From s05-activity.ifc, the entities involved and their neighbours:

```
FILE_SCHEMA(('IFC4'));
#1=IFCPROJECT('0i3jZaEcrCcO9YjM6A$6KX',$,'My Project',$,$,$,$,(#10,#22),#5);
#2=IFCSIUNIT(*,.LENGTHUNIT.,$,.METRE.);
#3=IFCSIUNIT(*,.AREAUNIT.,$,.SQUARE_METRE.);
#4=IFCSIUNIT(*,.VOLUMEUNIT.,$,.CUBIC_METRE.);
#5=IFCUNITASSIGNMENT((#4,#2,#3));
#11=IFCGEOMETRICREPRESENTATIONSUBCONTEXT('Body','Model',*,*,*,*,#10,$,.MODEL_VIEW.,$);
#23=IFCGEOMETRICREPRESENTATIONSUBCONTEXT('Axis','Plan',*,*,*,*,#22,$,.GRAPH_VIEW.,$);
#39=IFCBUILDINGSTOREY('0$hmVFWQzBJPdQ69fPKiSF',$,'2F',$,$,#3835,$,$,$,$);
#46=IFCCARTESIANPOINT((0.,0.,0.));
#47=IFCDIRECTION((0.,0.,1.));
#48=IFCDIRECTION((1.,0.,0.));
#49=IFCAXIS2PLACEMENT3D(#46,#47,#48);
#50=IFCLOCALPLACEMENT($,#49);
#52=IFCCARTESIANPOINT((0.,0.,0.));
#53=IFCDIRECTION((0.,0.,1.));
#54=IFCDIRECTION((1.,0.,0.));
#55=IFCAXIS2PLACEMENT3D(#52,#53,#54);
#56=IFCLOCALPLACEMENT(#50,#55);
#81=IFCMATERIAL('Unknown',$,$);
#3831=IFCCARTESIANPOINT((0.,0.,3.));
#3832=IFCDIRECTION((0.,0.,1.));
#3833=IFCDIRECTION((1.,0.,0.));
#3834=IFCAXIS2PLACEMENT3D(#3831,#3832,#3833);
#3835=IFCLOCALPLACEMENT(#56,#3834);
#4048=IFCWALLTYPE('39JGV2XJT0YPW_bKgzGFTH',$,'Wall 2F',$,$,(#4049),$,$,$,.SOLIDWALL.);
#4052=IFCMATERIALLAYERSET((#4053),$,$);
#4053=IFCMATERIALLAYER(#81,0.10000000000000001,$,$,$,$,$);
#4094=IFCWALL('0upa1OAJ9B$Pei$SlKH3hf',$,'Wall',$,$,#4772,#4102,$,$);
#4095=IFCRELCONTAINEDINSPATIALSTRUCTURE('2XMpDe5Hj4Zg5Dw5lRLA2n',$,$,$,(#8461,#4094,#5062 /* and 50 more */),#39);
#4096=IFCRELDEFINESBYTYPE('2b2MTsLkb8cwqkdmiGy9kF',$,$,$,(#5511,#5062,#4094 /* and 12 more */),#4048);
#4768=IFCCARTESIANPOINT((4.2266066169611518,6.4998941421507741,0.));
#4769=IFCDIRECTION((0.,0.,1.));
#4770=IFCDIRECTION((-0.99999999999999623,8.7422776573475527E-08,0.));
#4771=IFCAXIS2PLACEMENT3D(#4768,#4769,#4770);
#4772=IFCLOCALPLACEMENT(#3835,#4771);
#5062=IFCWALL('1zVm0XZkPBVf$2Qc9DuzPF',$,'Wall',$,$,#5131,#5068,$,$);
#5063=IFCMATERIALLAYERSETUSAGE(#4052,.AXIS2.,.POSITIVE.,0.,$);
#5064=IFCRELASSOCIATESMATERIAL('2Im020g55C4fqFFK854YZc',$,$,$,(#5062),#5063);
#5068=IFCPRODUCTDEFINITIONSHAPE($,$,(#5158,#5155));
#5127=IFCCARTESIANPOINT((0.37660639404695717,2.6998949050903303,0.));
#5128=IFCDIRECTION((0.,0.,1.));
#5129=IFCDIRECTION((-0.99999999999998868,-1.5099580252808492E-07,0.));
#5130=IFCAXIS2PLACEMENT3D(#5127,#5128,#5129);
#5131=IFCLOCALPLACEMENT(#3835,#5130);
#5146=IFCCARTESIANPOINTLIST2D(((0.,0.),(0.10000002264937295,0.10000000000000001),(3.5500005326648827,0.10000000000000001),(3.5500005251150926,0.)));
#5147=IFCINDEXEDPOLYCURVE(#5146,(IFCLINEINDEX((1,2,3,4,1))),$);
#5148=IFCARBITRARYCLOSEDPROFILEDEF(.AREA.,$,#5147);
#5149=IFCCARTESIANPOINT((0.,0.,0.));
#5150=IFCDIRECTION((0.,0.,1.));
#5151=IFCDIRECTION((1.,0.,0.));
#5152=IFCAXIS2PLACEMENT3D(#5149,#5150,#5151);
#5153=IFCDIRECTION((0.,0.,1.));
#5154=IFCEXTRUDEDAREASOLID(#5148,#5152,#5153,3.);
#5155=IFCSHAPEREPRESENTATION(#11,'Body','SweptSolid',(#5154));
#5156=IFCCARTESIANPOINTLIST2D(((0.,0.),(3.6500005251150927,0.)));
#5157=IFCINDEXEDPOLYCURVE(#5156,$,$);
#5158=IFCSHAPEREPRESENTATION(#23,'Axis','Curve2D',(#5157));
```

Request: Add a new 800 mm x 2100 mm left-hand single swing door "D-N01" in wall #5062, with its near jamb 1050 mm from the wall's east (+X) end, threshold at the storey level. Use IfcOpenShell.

```python
import numpy as np
import ifcopenshell
import ifcopenshell.api.feature
import ifcopenshell.api.geometry
import ifcopenshell.api.root
import ifcopenshell.api.spatial
import ifcopenshell.geom
import ifcopenshell.util.element
import ifcopenshell.util.placement
import ifcopenshell.util.representation
import ifcopenshell.util.shape
import ifcopenshell.util.unit

model = ifcopenshell.open("s05-activity.ifc")
unit_scale = ifcopenshell.util.unit.calculate_unit_scale(model)
settings = ifcopenshell.geom.settings()


def volume(element):
    """Net volume in cubic metres, openings subtracted."""
    shape = ifcopenshell.geom.create_shape(settings, element)
    return ifcopenshell.util.shape.get_volume(shape.geometry)


wall = model.by_id(5062)
storey = ifcopenshell.util.element.get_container(wall, ifc_class="IfcBuildingStorey")
context = ifcopenshell.util.representation.get_context(model, "Model", "Body", "MODEL_VIEW")
before = volume(wall)

width, height, from_end, sill = 0.8, 2.1, 1.05, 0.0  # metres

# The wall runs along its own X axis, and the end named is its -X end.
wall_shape = ifcopenshell.geom.create_shape(settings, wall)
x, y, z = ifcopenshell.util.shape.get_vertices(wall_shape.geometry).T
start = x.min() + from_end
face, thickness = float(y.min()), float(y.max() - y.min())
wall_matrix = ifcopenshell.util.placement.get_local_placement(wall.ObjectPlacement)
level = ifcopenshell.util.placement.get_local_placement(storey.ObjectPlacement)[2, 3]


def in_wall(x, y):
    """Placement at x, y metres in the wall's axes, at sill height."""
    matrix = wall_matrix.copy()
    matrix[:, 3] = wall_matrix @ np.array([x / unit_scale, y / unit_scale, 0.0, 1.0])
    matrix[2, 3] = level + sill / unit_scale
    return matrix


# Opening: a box that overshoots both wall faces by 50 mm.
opening = ifcopenshell.api.root.create_entity(model, ifc_class="IfcOpeningElement", predefined_type="OPENING")
box = ifcopenshell.api.geometry.add_wall_representation(
    model, context=context, length=width, height=height, thickness=thickness + 0.1
)
ifcopenshell.api.geometry.assign_representation(model, product=opening, representation=box)
ifcopenshell.api.geometry.edit_object_placement(model, product=opening, matrix=in_wall(start, face - 0.05), is_si=False)
ifcopenshell.api.feature.add_feature(model, feature=opening, element=wall)

door = ifcopenshell.api.root.create_entity(model, ifc_class="IfcDoor", name="D-N01", predefined_type="DOOR")
door.OverallWidth, door.OverallHeight = width / unit_scale, height / unit_scale
door.OperationType = "SINGLE_SWING_LEFT"
body = ifcopenshell.api.geometry.add_door_representation(
    model,
    context=context,
    overall_width=door.OverallWidth,
    overall_height=door.OverallHeight,
    operation_type="SINGLE_SWING_LEFT",
    lining_properties={"LiningDepth": thickness / unit_scale, "ThresholdDepth": thickness / unit_scale},
)
ifcopenshell.api.geometry.assign_representation(model, product=door, representation=body)
ifcopenshell.api.spatial.assign_container(model, products=[door], relating_structure=storey)
ifcopenshell.api.feature.add_filling(model, opening=opening, element=door)

# The lining spans the wall, so the door starts at the wall face.
ifcopenshell.api.geometry.edit_object_placement(model, product=door, matrix=in_wall(start, face), is_si=False)

after = volume(wall)

print(f"wall volume {before:.3f} -> {after:.3f} m3")

model.write("s05-activity_updated.ifc")
```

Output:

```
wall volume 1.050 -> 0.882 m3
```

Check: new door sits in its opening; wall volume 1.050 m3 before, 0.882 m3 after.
